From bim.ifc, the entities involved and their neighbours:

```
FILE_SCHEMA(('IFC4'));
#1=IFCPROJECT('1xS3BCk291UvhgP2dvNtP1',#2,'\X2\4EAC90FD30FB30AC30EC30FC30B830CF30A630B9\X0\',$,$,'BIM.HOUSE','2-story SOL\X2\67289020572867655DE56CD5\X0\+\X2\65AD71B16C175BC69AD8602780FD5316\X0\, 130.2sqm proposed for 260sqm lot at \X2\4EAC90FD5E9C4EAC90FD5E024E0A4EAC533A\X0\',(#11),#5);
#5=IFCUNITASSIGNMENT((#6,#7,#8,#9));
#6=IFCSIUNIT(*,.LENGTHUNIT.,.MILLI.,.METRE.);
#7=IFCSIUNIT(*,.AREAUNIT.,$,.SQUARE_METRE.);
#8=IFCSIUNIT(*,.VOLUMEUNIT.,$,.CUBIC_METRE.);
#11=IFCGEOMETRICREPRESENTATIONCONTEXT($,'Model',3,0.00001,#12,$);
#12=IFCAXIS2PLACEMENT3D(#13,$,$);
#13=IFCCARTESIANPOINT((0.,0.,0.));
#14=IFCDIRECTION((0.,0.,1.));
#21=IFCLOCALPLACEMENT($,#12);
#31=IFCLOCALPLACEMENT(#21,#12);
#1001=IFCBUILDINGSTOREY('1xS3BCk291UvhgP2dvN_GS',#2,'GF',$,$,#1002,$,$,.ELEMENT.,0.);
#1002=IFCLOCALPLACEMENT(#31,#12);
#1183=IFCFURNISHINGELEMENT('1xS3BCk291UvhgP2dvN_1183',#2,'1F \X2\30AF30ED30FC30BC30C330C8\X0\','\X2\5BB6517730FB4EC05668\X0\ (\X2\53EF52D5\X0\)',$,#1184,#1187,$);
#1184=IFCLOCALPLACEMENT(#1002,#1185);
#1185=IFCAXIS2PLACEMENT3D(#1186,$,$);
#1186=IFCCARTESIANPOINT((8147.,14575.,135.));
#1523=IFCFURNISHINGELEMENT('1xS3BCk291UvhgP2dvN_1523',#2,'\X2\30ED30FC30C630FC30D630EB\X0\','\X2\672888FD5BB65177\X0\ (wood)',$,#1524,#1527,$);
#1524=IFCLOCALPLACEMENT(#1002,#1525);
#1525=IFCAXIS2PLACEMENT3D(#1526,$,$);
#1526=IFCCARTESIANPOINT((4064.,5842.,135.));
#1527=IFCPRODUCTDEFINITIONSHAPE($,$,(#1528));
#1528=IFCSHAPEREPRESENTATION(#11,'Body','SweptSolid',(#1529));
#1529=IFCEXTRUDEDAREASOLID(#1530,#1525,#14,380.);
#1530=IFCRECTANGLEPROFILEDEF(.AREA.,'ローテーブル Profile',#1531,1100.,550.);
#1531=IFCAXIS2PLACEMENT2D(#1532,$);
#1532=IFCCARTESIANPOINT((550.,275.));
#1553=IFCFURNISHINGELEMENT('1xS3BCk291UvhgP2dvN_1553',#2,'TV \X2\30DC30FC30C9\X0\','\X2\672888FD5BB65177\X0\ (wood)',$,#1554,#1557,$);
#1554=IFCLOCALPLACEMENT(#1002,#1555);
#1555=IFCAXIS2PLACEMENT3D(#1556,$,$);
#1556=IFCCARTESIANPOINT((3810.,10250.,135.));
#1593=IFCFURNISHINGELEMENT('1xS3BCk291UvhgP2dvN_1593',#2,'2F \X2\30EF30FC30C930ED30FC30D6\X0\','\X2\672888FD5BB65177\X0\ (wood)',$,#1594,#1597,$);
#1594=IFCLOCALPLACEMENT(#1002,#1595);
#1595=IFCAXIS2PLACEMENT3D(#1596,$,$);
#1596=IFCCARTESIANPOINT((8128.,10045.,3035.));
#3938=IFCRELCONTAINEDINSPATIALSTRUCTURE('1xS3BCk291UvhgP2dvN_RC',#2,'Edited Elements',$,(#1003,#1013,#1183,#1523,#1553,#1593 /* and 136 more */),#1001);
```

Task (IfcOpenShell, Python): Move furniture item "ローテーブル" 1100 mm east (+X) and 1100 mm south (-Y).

```python
import ifcopenshell
import ifcopenshell.api.geometry
import ifcopenshell.util.placement
import ifcopenshell.util.unit

model = ifcopenshell.open("bim.ifc")
unit_scale = ifcopenshell.util.unit.calculate_unit_scale(model)

item = model.by_guid("1xS3BCk291UvhgP2dvN_1523")
matrix = ifcopenshell.util.placement.get_local_placement(item.ObjectPlacement)
matrix[0, 3] += 1.1 / unit_scale
matrix[1, 3] -= 1.1 / unit_scale
ifcopenshell.api.geometry.edit_object_placement(model, product=item, matrix=matrix, is_si=False)

print(ifcopenshell.util.placement.get_local_placement(item.ObjectPlacement).round(3) + 0.0)

model.write("bim-out.ifc")
```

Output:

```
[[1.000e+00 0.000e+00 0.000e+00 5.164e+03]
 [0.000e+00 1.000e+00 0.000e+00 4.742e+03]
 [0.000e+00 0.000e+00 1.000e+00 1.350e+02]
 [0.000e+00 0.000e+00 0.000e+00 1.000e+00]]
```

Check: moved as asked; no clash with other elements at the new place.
